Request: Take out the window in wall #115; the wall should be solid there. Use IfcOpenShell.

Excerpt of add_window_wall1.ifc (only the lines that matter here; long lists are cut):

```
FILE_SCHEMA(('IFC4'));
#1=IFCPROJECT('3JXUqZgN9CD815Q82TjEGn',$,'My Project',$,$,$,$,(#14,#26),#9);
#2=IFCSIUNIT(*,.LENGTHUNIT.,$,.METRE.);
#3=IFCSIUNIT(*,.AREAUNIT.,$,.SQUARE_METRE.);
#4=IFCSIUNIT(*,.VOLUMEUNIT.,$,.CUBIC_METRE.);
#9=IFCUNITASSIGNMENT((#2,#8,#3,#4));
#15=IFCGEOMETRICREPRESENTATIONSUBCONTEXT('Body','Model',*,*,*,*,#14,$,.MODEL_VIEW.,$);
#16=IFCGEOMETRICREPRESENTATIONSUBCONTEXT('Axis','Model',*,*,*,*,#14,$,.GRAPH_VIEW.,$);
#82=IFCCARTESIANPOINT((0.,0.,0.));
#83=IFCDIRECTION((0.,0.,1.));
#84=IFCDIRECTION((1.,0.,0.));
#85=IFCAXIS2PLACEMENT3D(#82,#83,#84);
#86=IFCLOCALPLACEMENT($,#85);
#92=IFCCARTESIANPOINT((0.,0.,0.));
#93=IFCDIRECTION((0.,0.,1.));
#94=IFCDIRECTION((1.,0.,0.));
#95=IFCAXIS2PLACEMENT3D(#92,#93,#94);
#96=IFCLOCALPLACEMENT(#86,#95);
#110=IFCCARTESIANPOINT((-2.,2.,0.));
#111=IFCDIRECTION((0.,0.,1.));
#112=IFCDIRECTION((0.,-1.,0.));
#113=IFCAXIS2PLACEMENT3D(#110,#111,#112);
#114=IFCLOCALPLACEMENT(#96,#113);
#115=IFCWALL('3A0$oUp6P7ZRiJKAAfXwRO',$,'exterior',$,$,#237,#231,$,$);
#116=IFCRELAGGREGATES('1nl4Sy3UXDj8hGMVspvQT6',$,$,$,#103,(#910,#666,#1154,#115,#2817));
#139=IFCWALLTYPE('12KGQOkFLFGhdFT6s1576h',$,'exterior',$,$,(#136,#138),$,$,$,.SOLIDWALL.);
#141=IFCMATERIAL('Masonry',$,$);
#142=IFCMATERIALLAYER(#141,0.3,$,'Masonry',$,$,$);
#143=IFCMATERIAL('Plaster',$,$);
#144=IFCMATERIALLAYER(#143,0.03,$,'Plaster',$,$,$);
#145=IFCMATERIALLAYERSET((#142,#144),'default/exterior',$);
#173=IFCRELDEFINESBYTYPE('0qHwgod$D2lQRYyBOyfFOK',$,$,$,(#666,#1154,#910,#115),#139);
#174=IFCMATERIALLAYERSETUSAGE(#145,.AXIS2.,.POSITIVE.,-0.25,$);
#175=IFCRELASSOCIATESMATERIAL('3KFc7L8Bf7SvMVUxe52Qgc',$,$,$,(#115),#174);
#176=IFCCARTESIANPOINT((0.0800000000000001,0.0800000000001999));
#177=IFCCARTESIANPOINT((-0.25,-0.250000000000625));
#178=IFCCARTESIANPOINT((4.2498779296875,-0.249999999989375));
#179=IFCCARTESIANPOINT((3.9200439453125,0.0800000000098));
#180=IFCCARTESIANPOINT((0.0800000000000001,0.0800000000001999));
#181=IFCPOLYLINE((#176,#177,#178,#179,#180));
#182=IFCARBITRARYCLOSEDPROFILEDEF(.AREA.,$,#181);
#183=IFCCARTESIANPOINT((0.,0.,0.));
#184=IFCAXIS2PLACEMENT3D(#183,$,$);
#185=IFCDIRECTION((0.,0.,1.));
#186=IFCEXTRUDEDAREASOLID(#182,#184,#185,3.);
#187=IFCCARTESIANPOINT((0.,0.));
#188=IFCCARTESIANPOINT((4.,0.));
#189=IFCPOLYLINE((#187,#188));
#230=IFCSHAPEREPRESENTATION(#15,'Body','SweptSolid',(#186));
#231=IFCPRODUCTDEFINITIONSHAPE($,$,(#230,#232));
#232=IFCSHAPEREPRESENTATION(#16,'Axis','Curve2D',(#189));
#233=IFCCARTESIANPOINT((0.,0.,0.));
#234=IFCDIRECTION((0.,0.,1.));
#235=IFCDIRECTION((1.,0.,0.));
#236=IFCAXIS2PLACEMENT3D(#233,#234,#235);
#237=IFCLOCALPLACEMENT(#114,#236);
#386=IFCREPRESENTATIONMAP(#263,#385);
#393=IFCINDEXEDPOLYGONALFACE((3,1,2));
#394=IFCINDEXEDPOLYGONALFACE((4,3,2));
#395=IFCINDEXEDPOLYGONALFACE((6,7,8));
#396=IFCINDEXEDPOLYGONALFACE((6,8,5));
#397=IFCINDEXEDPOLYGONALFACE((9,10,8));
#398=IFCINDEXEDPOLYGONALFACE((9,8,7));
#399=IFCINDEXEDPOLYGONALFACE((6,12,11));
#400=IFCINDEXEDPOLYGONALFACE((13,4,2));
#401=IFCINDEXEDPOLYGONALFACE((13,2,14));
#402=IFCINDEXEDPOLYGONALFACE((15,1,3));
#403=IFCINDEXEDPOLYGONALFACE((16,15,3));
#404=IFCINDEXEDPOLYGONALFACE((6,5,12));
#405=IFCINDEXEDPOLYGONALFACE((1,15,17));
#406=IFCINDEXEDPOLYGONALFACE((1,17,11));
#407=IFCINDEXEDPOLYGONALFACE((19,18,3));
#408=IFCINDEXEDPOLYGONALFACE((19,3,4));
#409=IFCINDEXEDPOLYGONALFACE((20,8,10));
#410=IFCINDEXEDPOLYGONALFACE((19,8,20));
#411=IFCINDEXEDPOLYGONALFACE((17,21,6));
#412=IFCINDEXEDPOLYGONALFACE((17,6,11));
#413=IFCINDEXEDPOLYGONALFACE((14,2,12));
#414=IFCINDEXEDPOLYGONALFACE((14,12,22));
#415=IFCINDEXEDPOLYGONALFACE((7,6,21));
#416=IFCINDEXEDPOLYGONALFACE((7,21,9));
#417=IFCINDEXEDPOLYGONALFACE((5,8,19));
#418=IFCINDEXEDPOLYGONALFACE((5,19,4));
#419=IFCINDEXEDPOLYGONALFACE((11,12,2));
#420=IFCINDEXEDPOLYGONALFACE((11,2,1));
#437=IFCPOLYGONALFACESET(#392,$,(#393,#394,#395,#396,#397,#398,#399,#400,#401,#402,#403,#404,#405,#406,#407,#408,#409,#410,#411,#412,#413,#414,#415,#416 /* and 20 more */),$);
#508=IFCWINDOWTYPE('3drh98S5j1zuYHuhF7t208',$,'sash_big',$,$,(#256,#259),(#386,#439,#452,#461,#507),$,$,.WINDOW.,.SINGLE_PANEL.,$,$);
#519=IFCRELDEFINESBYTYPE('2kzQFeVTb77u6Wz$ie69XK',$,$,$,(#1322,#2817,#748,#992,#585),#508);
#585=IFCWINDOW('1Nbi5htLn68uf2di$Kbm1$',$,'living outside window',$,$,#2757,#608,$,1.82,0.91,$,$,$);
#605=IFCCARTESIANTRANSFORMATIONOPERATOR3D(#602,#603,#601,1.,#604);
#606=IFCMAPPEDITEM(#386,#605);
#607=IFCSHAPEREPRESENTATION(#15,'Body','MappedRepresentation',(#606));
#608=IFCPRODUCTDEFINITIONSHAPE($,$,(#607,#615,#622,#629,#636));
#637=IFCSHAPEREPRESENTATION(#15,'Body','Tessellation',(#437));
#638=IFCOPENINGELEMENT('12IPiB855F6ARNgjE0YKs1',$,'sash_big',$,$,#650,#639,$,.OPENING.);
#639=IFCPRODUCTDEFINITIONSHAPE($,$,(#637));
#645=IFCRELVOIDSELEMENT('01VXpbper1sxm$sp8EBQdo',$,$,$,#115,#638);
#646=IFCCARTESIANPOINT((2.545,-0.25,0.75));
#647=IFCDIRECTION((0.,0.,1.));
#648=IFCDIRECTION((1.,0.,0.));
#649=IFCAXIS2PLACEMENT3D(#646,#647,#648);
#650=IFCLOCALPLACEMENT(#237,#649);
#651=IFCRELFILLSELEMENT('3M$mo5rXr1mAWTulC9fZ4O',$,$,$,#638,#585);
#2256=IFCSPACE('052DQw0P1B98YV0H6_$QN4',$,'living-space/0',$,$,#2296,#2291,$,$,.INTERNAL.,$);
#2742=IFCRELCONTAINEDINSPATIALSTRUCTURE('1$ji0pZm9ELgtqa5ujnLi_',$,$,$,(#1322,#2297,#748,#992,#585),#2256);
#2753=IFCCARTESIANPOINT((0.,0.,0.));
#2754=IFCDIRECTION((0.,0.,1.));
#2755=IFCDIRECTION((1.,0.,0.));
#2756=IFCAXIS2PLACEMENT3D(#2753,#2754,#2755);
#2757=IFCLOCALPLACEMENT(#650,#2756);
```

```python
import ifcopenshell
import ifcopenshell.api.feature
import ifcopenshell.api.root
import ifcopenshell.geom
import ifcopenshell.util.shape

model = ifcopenshell.open("add_window_wall1.ifc")
settings = ifcopenshell.geom.settings()


def volume(element):
    """Net volume in cubic metres, openings subtracted."""
    shape = ifcopenshell.geom.create_shape(settings, element)
    return ifcopenshell.util.shape.get_volume(shape.geometry)


window = model.by_guid("1Nbi5htLn68uf2di$Kbm1$")
opening = window.FillsVoids[0].RelatingOpeningElement
wall = opening.VoidsElements[0].RelatingBuildingElement
before = volume(wall)

ifcopenshell.api.root.remove_product(model, product=window)
ifcopenshell.api.feature.remove_feature(model, feature=opening)

after = volume(wall)

print(f"wall volume {before:.3f} -> {after:.3f} m3")

model.write("add_window_wall1_edited.ifc")
```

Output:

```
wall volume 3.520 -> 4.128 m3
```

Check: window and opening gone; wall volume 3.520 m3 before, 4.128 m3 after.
